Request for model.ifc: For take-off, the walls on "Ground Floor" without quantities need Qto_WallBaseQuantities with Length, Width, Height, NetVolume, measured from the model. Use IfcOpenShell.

First a look at what the model holds.

```python
import ifcopenshell
import ifcopenshell.util.element
import ifcopenshell.util.unit

model = ifcopenshell.open("model.ifc")
print(model.schema)
for unit_type in ("LENGTHUNIT", "AREAUNIT", "VOLUMEUNIT"):
    print(unit_type, ifcopenshell.util.unit.calculate_unit_scale(model, unit_type))
storey = next(s for s in model.by_type("IfcBuildingStorey") if s.Name == "Ground Floor")
walls = [e for e in ifcopenshell.util.element.get_decomposition(storey) if e.is_a("IfcWall")]
for e in sorted(walls, key=lambda e: e.id()):
    print(e.id(), e.is_a(), e.Name, list(ifcopenshell.util.element.get_psets(e, qtos_only=True)), sep=" | ")
```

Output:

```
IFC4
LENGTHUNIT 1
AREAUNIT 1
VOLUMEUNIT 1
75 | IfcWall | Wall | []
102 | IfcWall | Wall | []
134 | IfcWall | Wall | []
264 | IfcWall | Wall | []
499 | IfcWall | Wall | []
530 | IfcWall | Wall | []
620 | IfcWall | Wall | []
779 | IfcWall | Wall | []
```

```python
import ifcopenshell
import ifcopenshell.api.pset
import ifcopenshell.geom
import ifcopenshell.util.element
import ifcopenshell.util.shape
import ifcopenshell.util.unit

model = ifcopenshell.open("model.ifc")
unit_scale = ifcopenshell.util.unit.calculate_unit_scale(model)
volume_scale = ifcopenshell.util.unit.calculate_unit_scale(model, "VOLUMEUNIT")
settings = ifcopenshell.geom.settings()

storey = next(s for s in model.by_type("IfcBuildingStorey") if s.Name == "Ground Floor")
walls = [e for e in ifcopenshell.util.element.get_decomposition(storey) if e.is_a("IfcWall")]

for e in sorted(walls, key=lambda e: e.id()):
    if ifcopenshell.util.element.get_psets(e, qtos_only=True, should_inherit=False):
        continue
    # Geometry comes back in metres, in the element's own axes.
    shape = ifcopenshell.geom.create_shape(settings, e)
    values = {
        "Length": ifcopenshell.util.shape.get_x(shape.geometry) / unit_scale,
        "Width": ifcopenshell.util.shape.get_y(shape.geometry) / unit_scale,
        "Height": ifcopenshell.util.shape.get_z(shape.geometry) / unit_scale,
        "NetVolume": ifcopenshell.util.shape.get_volume(shape.geometry) / volume_scale,
    }
    qto = ifcopenshell.api.pset.add_qto(model, product=e, name="Qto_WallBaseQuantities")
    ifcopenshell.api.pset.edit_qto(model, qto=qto, properties=values)
    print(e.id(), {k: round(v, 3) for k, v in values.items()})

model.write("model_updated.ifc")
```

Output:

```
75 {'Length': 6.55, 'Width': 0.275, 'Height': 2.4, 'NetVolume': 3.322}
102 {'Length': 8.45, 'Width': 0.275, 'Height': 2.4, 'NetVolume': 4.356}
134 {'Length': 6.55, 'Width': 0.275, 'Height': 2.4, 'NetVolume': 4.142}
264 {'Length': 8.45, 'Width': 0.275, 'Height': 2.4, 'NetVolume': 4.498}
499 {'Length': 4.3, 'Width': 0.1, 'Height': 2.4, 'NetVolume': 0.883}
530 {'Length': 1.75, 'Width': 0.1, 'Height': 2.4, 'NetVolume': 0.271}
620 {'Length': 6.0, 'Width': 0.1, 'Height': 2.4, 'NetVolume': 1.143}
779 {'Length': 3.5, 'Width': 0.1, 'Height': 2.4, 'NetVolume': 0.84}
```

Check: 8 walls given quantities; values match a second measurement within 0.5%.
